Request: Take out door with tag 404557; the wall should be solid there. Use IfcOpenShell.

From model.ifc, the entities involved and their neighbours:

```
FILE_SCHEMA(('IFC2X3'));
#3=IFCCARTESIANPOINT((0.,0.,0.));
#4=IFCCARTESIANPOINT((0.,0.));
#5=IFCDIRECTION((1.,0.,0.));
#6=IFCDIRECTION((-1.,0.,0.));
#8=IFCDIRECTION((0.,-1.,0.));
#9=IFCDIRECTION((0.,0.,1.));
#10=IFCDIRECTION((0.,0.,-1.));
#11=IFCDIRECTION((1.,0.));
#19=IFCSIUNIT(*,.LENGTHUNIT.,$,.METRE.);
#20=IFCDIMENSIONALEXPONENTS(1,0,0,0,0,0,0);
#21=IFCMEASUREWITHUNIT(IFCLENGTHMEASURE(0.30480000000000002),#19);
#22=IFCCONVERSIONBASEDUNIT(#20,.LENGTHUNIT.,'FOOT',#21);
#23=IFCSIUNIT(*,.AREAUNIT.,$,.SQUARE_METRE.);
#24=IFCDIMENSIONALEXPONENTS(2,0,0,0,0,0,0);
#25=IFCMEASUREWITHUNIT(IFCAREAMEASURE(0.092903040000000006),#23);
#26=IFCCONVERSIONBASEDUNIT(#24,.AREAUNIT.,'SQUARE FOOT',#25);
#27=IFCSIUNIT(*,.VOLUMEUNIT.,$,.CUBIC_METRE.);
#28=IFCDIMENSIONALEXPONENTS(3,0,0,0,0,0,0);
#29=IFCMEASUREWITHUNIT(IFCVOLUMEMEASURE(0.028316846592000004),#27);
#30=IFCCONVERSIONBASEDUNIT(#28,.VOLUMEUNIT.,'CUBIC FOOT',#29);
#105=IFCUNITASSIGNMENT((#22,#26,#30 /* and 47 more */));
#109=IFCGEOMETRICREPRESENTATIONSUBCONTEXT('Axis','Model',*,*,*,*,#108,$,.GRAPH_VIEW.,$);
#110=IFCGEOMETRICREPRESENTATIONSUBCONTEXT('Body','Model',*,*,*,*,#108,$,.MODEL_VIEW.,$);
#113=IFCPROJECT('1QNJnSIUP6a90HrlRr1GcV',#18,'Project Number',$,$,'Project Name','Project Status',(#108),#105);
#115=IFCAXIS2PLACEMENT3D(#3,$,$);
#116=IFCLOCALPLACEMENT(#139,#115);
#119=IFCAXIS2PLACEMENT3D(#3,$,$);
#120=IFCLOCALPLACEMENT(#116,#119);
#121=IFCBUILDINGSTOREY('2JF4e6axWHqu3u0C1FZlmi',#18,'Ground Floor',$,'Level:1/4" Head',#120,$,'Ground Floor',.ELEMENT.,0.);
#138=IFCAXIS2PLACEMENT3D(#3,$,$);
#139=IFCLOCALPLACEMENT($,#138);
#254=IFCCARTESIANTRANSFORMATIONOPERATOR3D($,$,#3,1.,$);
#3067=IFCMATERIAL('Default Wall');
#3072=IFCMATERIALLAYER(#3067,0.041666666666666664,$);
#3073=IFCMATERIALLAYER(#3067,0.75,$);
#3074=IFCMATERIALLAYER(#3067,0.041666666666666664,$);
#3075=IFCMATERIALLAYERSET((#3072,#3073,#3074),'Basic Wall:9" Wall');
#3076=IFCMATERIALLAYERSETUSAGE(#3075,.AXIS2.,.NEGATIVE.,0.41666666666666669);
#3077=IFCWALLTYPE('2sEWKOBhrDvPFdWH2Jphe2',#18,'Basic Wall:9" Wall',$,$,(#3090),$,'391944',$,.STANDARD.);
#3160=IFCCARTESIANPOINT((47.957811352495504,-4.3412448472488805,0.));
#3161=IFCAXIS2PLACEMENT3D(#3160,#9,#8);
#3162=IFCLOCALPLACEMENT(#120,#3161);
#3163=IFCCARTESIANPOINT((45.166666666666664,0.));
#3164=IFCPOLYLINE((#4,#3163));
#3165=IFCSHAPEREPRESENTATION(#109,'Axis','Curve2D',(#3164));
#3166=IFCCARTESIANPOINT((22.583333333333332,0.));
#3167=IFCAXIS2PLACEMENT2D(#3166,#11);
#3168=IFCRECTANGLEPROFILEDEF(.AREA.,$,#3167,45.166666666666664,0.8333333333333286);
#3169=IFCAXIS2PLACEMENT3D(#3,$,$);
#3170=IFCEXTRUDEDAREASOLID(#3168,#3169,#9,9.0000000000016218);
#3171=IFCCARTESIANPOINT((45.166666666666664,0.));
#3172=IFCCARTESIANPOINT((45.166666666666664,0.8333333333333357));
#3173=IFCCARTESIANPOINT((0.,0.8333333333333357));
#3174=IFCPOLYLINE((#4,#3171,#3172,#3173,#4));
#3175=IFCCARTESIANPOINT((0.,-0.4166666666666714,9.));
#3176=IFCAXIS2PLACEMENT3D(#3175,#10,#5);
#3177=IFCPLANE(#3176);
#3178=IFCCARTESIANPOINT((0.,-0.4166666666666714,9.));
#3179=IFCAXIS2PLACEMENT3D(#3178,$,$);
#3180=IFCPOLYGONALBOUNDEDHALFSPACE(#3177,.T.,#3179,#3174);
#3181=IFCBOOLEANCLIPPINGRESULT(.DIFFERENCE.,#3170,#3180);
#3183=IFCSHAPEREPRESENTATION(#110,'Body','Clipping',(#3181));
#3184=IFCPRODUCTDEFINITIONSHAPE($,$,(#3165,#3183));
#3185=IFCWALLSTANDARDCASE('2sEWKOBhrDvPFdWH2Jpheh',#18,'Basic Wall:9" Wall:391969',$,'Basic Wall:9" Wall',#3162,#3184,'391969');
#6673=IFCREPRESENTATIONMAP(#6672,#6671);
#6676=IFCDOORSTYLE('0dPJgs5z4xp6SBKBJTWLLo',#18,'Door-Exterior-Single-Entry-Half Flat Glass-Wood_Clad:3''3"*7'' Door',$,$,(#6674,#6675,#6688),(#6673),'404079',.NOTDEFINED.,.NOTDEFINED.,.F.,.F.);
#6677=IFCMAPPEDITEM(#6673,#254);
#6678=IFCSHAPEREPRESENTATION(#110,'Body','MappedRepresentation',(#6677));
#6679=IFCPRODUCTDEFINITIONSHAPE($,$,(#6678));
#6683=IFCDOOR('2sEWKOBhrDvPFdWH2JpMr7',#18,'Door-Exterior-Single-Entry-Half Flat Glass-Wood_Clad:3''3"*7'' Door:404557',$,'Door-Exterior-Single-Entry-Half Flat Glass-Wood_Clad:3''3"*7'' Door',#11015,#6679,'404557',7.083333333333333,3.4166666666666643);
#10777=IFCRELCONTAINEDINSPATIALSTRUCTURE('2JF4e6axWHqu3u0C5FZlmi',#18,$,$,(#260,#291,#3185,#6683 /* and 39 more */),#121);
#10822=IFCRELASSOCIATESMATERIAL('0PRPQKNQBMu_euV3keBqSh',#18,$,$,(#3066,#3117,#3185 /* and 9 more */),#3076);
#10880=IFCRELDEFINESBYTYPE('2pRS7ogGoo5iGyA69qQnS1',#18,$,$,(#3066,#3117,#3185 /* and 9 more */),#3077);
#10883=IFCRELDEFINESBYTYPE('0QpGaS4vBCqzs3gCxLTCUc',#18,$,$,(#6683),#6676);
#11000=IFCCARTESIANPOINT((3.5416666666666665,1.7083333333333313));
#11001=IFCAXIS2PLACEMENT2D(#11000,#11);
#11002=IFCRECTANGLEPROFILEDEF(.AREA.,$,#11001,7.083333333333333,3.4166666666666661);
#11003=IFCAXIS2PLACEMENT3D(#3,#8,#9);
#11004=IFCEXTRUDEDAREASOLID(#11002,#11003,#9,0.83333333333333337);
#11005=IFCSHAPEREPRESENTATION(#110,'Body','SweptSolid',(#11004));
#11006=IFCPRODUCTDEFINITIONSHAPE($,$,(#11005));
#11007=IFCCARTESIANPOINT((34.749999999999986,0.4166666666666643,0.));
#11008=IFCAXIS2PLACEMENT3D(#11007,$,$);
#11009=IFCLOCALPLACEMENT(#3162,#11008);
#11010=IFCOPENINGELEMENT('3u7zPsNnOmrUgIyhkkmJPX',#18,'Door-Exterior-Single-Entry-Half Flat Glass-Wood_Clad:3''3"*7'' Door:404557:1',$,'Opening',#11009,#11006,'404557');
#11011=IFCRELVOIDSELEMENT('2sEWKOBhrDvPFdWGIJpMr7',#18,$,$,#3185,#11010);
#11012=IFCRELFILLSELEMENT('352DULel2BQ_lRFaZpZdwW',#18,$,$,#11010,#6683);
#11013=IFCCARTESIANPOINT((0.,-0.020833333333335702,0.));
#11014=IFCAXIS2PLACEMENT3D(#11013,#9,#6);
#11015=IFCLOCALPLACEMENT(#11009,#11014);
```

```python
import ifcopenshell
import ifcopenshell.api.feature
import ifcopenshell.api.root
import ifcopenshell.geom
import ifcopenshell.util.shape

model = ifcopenshell.open("model.ifc")
settings = ifcopenshell.geom.settings()


def volume(element):
    """Net volume in cubic metres, openings subtracted."""
    shape = ifcopenshell.geom.create_shape(settings, element)
    return ifcopenshell.util.shape.get_volume(shape.geometry)


door = model.by_guid("2sEWKOBhrDvPFdWH2JpMr7")
opening = door.FillsVoids[0].RelatingOpeningElement
wall = opening.VoidsElements[0].RelatingBuildingElement
before = volume(wall)

ifcopenshell.api.root.remove_product(model, product=door)
ifcopenshell.api.feature.remove_feature(model, feature=opening)

after = volume(wall)

print(f"wall volume {before:.3f} -> {after:.3f} m3")

model.write("model_rev.ifc")
```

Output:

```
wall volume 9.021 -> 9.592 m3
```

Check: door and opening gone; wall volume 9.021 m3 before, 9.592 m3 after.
